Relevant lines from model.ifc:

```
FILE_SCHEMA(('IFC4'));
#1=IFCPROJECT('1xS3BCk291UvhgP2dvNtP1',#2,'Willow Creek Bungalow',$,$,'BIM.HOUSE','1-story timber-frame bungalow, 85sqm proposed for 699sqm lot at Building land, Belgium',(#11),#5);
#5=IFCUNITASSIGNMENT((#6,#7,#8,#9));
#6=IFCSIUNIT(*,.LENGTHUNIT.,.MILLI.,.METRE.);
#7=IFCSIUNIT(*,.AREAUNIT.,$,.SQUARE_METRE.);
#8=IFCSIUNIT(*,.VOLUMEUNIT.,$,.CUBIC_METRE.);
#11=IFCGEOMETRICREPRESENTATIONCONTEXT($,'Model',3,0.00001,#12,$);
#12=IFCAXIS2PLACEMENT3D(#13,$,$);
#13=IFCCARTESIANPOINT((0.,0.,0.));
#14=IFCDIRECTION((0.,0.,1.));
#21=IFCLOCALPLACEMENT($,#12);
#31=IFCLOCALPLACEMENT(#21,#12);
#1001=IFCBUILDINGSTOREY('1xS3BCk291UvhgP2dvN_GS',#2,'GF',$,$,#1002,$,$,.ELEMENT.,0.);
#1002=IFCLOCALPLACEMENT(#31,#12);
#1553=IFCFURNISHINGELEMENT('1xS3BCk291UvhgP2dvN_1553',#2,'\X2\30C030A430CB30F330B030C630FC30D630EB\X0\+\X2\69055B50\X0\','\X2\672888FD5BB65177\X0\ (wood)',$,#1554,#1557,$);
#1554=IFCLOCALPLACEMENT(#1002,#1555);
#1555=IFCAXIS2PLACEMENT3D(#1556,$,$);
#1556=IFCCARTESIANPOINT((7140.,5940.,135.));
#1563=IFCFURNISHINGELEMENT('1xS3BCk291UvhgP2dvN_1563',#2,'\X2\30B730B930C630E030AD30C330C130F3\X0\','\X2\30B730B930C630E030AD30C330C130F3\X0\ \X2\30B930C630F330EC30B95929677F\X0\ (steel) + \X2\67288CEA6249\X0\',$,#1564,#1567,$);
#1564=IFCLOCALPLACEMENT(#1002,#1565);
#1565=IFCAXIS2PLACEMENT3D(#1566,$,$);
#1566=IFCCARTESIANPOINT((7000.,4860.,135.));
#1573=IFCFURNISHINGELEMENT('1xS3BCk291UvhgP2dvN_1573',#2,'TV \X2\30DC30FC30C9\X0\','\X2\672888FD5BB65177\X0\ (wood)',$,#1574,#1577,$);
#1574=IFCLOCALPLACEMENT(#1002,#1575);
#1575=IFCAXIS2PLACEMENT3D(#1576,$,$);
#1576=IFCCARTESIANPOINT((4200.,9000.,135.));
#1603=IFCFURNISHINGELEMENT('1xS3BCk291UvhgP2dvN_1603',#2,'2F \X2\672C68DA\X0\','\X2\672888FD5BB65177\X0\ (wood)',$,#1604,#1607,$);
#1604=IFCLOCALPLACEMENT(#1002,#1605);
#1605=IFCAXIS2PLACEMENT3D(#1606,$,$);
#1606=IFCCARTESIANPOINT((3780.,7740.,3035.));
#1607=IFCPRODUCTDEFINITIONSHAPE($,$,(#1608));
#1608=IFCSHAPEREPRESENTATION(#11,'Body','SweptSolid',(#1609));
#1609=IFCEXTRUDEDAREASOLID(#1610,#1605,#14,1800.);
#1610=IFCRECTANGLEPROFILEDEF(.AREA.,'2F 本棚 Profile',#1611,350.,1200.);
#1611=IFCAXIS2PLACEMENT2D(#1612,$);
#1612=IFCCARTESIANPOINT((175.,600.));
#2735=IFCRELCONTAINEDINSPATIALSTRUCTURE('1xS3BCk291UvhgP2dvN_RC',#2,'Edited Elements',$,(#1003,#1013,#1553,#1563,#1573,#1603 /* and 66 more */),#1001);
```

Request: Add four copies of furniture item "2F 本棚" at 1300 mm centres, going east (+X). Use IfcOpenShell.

```python
import numpy as np
import ifcopenshell
import ifcopenshell.api.geometry
import ifcopenshell.api.root
import ifcopenshell.util.element
import ifcopenshell.util.placement
import ifcopenshell.util.unit

model = ifcopenshell.open("model.ifc")
unit_scale = ifcopenshell.util.unit.calculate_unit_scale(model)


def reuse_history(source, copy):
    """copy_class also copies each property set's owner history, people and application; keep the originals."""
    for rel in copy.IsDefinedBy:
        if rel.is_a("IfcRelDefinesByProperties") and (history := rel.RelatingPropertyDefinition.OwnerHistory):
            rel.RelatingPropertyDefinition.OwnerHistory = source.OwnerHistory
            ifcopenshell.util.element.remove_deep2(model, history)


source = model.by_guid("1xS3BCk291UvhgP2dvN_1603")
base = ifcopenshell.util.placement.get_local_placement(source.ObjectPlacement)
step = np.array([1.0, 0.0, 0.0]) * 1.3 / unit_scale

for i in range(1, 5):
    copy = ifcopenshell.api.root.copy_class(model, product=source)
    copy.Representation = ifcopenshell.util.element.copy_deep(
        model, source.Representation, exclude=["IfcGeometricRepresentationContext", "IfcRepresentationMap"]
    )
    reuse_history(source, copy)
    matrix = base.copy()
    matrix[:3, 3] += i * step
    print("added at", matrix[:3, 3].round(3) + 0.0)
    ifcopenshell.api.geometry.edit_object_placement(model, product=copy, matrix=matrix, is_si=False)

model.write("model_updated.ifc")
```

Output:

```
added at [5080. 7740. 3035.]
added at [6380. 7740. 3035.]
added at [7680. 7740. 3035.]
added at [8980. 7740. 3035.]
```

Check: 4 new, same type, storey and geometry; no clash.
